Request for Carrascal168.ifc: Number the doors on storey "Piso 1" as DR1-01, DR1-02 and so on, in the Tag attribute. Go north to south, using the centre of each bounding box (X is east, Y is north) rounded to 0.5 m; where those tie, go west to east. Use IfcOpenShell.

First a look at what the model holds.

```python
import ifcopenshell
import ifcopenshell.util.element
import ifcopenshell.util.placement

model = ifcopenshell.open("Carrascal168.ifc")
print(model.schema)
storey = next(s for s in model.by_type("IfcBuildingStorey") if s.Name == "Piso 1")
doors = [e for e in ifcopenshell.util.element.get_decomposition(storey) if e.is_a("IfcDoor")]
for e in sorted(doors, key=lambda e: e.id()):
    origin = ifcopenshell.util.placement.get_local_placement(e.ObjectPlacement)[:3, 3]
    print(e.id(), e.Tag, e.Name, origin.round(2) + 0.0, sep=" | ")
```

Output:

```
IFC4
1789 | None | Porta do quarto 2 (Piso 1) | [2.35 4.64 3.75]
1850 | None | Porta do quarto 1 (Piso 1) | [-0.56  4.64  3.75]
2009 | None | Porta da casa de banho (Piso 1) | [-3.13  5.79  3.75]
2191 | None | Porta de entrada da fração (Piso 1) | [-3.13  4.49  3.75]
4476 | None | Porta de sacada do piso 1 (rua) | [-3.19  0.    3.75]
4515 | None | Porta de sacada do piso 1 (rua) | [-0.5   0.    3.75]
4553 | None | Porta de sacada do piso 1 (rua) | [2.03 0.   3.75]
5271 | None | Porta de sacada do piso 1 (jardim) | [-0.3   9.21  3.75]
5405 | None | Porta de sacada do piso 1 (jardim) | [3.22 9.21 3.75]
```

```python
import ifcopenshell
import ifcopenshell.geom
import ifcopenshell.util.element
import ifcopenshell.util.shape

model = ifcopenshell.open("Carrascal168.ifc")
settings = ifcopenshell.geom.settings()
settings.set("use-world-coords", True)


def centre(element):
    shape = ifcopenshell.geom.create_shape(settings, element)
    return ifcopenshell.util.shape.get_bbox_centroid(shape.geometry)


storey = next(s for s in model.by_type("IfcBuildingStorey") if s.Name == "Piso 1")
doors = [e for e in ifcopenshell.util.element.get_decomposition(storey) if e.is_a("IfcDoor")]

# Insertion points can sit at a corner or the storey origin, so sort by the geometry (in metres).
centres = {e: centre(e) for e in doors}
doors.sort(key=lambda e: (-round(centres[e][1] / 0.5), centres[e][0]))

for i, e in enumerate(doors, start=1):
    number = f"DR1-{i:02d}"
    e.Tag = number
    print(e.id(), number)

model.write("Carrascal168_v2.ifc")
```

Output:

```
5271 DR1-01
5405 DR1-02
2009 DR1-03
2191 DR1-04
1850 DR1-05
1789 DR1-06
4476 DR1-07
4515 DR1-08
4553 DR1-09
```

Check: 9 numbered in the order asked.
